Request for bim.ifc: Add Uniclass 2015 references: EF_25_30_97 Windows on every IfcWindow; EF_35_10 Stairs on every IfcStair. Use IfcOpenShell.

First a look at what the model holds.

```python
import ifcopenshell

model = ifcopenshell.open("bim.ifc")
print(model.schema)
print("classifications:", [c.Name for c in model.by_type("IfcClassification")])
for ifc_class in ("IfcDoor", "IfcRoof", "IfcStair", "IfcWall", "IfcWindow"):
    print(ifc_class, len(model.by_type(ifc_class)))
```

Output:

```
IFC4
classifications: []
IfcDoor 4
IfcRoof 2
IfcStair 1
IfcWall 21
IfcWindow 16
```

```python
import ifcopenshell
import ifcopenshell.api.classification

model = ifcopenshell.open("bim.ifc")

system = ifcopenshell.api.classification.add_classification(model, classification="Uniclass 2015")

codes = {
    "IfcWindow": ("EF_25_30_97", "Windows"),
    "IfcStair": ("EF_35_10", "Stairs"),
}
for ifc_class, (code, name) in codes.items():
    products = model.by_type(ifc_class)
    ifcopenshell.api.classification.add_reference(
        model, products=products, classification=system, identification=code, name=name
    )
    print(code, len(products))

model.write("bim_rev.ifc")
```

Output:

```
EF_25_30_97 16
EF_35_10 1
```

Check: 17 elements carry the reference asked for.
